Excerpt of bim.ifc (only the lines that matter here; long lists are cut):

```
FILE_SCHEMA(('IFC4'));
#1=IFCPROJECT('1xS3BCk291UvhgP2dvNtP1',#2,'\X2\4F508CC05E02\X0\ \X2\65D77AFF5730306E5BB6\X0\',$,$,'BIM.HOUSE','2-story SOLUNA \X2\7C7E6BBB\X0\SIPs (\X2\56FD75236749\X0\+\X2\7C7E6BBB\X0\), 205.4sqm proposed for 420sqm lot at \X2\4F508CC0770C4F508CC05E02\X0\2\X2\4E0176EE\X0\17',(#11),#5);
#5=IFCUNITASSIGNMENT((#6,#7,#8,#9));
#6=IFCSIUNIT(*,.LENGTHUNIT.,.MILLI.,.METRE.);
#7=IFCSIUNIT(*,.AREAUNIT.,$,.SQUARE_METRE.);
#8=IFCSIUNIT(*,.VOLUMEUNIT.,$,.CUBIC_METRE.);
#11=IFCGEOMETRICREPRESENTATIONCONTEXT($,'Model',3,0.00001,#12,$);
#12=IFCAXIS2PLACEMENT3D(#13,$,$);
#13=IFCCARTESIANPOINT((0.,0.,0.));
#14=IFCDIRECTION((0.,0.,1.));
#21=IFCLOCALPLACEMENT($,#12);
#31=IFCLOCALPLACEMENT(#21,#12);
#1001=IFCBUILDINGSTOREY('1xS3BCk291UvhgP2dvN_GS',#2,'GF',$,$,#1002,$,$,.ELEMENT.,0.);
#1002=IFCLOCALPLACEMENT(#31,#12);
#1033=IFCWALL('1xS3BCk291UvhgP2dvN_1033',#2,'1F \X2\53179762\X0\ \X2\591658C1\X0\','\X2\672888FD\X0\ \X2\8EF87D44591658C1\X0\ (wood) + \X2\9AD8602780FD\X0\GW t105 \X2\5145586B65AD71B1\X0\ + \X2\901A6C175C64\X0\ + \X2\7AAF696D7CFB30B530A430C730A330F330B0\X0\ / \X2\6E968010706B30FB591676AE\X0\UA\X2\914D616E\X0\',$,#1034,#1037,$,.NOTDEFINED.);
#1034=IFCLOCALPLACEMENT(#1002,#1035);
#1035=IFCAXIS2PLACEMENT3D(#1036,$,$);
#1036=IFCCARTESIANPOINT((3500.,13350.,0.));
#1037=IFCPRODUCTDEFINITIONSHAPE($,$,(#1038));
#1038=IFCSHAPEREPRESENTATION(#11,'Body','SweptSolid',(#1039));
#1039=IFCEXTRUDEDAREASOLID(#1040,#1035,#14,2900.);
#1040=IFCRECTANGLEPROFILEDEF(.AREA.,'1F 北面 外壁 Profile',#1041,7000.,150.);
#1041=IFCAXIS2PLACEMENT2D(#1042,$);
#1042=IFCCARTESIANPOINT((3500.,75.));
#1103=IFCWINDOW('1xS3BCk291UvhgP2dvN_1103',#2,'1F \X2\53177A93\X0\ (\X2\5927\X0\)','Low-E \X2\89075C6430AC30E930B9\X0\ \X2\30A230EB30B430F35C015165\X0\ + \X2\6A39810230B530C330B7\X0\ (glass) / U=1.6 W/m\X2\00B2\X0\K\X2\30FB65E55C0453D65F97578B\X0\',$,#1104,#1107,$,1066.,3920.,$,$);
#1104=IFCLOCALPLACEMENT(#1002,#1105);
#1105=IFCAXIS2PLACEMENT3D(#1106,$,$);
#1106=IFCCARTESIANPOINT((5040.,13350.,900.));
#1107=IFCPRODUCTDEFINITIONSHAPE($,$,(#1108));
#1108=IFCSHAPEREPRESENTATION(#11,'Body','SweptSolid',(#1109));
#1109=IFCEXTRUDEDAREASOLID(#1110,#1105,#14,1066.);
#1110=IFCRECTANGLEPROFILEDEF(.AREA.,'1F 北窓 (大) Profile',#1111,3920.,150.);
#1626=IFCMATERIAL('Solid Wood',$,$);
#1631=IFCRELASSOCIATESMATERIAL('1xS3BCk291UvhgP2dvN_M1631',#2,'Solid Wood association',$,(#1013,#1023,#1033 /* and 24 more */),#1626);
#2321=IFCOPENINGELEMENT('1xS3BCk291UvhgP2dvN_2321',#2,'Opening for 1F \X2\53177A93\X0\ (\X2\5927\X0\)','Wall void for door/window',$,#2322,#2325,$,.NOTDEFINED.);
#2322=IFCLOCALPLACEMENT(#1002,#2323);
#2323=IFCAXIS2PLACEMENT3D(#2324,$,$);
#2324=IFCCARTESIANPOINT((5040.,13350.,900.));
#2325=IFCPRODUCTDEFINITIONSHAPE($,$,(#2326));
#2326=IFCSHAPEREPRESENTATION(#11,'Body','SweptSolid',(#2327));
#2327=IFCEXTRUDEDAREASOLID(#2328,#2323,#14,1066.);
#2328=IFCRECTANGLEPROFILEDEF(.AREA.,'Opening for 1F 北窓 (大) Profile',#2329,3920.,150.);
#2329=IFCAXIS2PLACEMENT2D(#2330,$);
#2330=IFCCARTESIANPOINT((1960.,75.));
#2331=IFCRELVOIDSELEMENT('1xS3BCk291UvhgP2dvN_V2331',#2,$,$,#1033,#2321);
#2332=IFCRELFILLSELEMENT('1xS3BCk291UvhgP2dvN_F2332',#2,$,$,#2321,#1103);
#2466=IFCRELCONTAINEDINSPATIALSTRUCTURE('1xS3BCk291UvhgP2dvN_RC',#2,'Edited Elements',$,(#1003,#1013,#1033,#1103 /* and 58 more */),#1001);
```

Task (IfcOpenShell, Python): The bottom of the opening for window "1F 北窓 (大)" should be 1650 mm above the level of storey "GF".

```python
import numpy as np
import ifcopenshell
import ifcopenshell.api.geometry
import ifcopenshell.geom
import ifcopenshell.util.element
import ifcopenshell.util.placement
import ifcopenshell.util.shape
import ifcopenshell.util.unit

model = ifcopenshell.open("bim.ifc")
unit_scale = ifcopenshell.util.unit.calculate_unit_scale(model)

window = model.by_guid("1xS3BCk291UvhgP2dvN_1103")
opening = window.FillsVoids[0].RelatingOpeningElement
storey = ifcopenshell.util.element.get_container(window, ifc_class="IfcBuildingStorey")
level = ifcopenshell.util.placement.get_local_placement(storey.ObjectPlacement)[2, 3]

# The opening's origin need not be at the sill, so measure its lowest point.
shape = ifcopenshell.geom.create_shape(ifcopenshell.geom.settings(), opening)
bottom = ifcopenshell.util.shape.get_shape_bottom_elevation(shape, shape.geometry) / unit_scale
dz = level + 1650.0 - bottom

shift = np.array([0.0, 0.0, dz])
# The window is not placed relative to its opening, so move both.
for product in (opening, window):
    matrix = ifcopenshell.util.placement.get_local_placement(product.ObjectPlacement)
    matrix[:3, 3] += shift
    ifcopenshell.api.geometry.edit_object_placement(model, product=product, matrix=matrix, is_si=False)

print(f"moved by {dz * unit_scale:+.3f} m")

model.write("bim_v2.ifc")
```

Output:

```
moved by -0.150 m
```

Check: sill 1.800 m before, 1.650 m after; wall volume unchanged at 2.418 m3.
